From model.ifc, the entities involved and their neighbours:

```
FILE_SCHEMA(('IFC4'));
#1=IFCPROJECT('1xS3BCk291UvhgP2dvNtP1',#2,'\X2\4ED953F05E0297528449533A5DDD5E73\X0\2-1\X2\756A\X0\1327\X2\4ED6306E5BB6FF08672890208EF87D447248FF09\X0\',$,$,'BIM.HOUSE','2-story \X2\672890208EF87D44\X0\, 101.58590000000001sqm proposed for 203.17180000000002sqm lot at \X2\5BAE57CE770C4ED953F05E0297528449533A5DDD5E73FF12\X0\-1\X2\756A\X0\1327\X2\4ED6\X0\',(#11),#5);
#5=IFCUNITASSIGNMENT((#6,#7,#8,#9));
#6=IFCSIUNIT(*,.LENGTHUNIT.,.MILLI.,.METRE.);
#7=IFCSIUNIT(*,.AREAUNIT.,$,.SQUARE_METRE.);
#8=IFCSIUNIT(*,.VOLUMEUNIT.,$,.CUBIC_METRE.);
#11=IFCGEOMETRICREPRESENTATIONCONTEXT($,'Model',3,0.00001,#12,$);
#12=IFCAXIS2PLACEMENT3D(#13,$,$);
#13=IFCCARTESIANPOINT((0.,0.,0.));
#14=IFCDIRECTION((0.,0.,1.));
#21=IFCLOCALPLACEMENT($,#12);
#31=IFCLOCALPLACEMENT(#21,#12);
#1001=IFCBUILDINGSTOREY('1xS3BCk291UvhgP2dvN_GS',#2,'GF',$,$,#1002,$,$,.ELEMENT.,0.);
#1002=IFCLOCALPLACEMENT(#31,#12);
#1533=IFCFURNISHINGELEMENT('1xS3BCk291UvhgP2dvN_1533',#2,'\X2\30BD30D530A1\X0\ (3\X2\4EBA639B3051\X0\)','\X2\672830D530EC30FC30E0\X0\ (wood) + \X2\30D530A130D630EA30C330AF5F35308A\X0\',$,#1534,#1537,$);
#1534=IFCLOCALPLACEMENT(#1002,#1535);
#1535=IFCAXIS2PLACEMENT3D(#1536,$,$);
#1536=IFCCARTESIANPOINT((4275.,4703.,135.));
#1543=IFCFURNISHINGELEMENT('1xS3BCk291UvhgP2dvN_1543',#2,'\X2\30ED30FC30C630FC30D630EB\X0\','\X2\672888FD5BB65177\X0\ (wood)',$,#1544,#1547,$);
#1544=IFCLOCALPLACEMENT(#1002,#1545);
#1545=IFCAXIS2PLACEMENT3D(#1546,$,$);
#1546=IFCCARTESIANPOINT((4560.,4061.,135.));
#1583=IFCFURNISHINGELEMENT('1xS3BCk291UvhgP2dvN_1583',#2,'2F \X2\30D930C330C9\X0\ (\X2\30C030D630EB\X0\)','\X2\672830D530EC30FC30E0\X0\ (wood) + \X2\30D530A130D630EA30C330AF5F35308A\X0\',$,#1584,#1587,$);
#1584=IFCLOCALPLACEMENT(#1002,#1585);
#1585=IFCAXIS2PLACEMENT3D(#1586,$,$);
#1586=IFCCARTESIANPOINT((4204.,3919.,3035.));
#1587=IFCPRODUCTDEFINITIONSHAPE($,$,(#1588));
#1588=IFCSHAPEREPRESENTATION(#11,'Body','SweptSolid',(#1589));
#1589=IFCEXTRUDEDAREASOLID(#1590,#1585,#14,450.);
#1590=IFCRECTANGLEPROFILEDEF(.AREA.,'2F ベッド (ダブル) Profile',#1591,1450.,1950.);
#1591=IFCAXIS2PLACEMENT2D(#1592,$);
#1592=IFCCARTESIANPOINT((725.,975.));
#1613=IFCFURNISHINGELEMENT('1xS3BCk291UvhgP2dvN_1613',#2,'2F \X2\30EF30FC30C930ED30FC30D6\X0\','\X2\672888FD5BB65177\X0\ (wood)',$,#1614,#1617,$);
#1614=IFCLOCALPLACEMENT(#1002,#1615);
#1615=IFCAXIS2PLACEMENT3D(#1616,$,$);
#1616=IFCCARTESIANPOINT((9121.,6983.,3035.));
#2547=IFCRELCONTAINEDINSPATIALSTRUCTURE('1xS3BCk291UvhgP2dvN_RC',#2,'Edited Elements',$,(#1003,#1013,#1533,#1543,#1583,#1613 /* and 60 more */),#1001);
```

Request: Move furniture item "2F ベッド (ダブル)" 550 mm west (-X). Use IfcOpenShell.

```python
import ifcopenshell
import ifcopenshell.api.geometry
import ifcopenshell.util.placement
import ifcopenshell.util.unit

model = ifcopenshell.open("model.ifc")
unit_scale = ifcopenshell.util.unit.calculate_unit_scale(model)

item = model.by_guid("1xS3BCk291UvhgP2dvN_1583")
matrix = ifcopenshell.util.placement.get_local_placement(item.ObjectPlacement)
matrix[0, 3] -= 0.55 / unit_scale
ifcopenshell.api.geometry.edit_object_placement(model, product=item, matrix=matrix, is_si=False)

print(ifcopenshell.util.placement.get_local_placement(item.ObjectPlacement).round(3) + 0.0)

model.write("model_rev.ifc")
```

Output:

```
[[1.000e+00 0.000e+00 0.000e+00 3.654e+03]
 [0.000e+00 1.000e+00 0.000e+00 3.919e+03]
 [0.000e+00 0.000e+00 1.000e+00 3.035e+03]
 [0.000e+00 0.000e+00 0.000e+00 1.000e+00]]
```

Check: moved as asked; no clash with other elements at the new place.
